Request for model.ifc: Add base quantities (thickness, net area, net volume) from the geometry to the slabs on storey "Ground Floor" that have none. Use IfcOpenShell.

First a look at what the model holds.

```python
import ifcopenshell
import ifcopenshell.util.element
import ifcopenshell.util.unit

model = ifcopenshell.open("model.ifc")
print(model.schema)
for unit_type in ("LENGTHUNIT", "AREAUNIT", "VOLUMEUNIT"):
    print(unit_type, ifcopenshell.util.unit.calculate_unit_scale(model, unit_type))
storey = next(s for s in model.by_type("IfcBuildingStorey") if s.Name == "Ground Floor")
slabs = [e for e in ifcopenshell.util.element.get_decomposition(storey) if e.is_a("IfcSlab")]
for e in sorted(slabs, key=lambda e: e.id()):
    print(e.id(), e.is_a(), e.Name, list(ifcopenshell.util.element.get_psets(e, qtos_only=True)), sep=" | ")
```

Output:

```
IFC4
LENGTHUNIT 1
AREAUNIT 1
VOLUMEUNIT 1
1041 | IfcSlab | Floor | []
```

```python
import ifcopenshell
import ifcopenshell.api.pset
import ifcopenshell.geom
import ifcopenshell.util.element
import ifcopenshell.util.shape
import ifcopenshell.util.unit

model = ifcopenshell.open("model.ifc")
unit_scale = ifcopenshell.util.unit.calculate_unit_scale(model)
area_scale = ifcopenshell.util.unit.calculate_unit_scale(model, "AREAUNIT")
volume_scale = ifcopenshell.util.unit.calculate_unit_scale(model, "VOLUMEUNIT")
settings = ifcopenshell.geom.settings()

storey = next(s for s in model.by_type("IfcBuildingStorey") if s.Name == "Ground Floor")
slabs = [e for e in ifcopenshell.util.element.get_decomposition(storey) if e.is_a("IfcSlab")]

for e in sorted(slabs, key=lambda e: e.id()):
    if ifcopenshell.util.element.get_psets(e, qtos_only=True, should_inherit=False):
        continue
    # Geometry comes back in metres, in the element's own axes.
    shape = ifcopenshell.geom.create_shape(settings, e)
    values = {
        "Width": ifcopenshell.util.shape.get_z(shape.geometry) / unit_scale,
        "NetArea": ifcopenshell.util.shape.get_footprint_area(shape.geometry) / area_scale,
        "NetVolume": ifcopenshell.util.shape.get_volume(shape.geometry) / volume_scale,
    }
    qto = ifcopenshell.api.pset.add_qto(model, product=e, name="Qto_SlabBaseQuantities")
    ifcopenshell.api.pset.edit_qto(model, qto=qto, properties=values)
    print(e.id(), {k: round(v, 3) for k, v in values.items()})

model.write("model_updated.ifc")
```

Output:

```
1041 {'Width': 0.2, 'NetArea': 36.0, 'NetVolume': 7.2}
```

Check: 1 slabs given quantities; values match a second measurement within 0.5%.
